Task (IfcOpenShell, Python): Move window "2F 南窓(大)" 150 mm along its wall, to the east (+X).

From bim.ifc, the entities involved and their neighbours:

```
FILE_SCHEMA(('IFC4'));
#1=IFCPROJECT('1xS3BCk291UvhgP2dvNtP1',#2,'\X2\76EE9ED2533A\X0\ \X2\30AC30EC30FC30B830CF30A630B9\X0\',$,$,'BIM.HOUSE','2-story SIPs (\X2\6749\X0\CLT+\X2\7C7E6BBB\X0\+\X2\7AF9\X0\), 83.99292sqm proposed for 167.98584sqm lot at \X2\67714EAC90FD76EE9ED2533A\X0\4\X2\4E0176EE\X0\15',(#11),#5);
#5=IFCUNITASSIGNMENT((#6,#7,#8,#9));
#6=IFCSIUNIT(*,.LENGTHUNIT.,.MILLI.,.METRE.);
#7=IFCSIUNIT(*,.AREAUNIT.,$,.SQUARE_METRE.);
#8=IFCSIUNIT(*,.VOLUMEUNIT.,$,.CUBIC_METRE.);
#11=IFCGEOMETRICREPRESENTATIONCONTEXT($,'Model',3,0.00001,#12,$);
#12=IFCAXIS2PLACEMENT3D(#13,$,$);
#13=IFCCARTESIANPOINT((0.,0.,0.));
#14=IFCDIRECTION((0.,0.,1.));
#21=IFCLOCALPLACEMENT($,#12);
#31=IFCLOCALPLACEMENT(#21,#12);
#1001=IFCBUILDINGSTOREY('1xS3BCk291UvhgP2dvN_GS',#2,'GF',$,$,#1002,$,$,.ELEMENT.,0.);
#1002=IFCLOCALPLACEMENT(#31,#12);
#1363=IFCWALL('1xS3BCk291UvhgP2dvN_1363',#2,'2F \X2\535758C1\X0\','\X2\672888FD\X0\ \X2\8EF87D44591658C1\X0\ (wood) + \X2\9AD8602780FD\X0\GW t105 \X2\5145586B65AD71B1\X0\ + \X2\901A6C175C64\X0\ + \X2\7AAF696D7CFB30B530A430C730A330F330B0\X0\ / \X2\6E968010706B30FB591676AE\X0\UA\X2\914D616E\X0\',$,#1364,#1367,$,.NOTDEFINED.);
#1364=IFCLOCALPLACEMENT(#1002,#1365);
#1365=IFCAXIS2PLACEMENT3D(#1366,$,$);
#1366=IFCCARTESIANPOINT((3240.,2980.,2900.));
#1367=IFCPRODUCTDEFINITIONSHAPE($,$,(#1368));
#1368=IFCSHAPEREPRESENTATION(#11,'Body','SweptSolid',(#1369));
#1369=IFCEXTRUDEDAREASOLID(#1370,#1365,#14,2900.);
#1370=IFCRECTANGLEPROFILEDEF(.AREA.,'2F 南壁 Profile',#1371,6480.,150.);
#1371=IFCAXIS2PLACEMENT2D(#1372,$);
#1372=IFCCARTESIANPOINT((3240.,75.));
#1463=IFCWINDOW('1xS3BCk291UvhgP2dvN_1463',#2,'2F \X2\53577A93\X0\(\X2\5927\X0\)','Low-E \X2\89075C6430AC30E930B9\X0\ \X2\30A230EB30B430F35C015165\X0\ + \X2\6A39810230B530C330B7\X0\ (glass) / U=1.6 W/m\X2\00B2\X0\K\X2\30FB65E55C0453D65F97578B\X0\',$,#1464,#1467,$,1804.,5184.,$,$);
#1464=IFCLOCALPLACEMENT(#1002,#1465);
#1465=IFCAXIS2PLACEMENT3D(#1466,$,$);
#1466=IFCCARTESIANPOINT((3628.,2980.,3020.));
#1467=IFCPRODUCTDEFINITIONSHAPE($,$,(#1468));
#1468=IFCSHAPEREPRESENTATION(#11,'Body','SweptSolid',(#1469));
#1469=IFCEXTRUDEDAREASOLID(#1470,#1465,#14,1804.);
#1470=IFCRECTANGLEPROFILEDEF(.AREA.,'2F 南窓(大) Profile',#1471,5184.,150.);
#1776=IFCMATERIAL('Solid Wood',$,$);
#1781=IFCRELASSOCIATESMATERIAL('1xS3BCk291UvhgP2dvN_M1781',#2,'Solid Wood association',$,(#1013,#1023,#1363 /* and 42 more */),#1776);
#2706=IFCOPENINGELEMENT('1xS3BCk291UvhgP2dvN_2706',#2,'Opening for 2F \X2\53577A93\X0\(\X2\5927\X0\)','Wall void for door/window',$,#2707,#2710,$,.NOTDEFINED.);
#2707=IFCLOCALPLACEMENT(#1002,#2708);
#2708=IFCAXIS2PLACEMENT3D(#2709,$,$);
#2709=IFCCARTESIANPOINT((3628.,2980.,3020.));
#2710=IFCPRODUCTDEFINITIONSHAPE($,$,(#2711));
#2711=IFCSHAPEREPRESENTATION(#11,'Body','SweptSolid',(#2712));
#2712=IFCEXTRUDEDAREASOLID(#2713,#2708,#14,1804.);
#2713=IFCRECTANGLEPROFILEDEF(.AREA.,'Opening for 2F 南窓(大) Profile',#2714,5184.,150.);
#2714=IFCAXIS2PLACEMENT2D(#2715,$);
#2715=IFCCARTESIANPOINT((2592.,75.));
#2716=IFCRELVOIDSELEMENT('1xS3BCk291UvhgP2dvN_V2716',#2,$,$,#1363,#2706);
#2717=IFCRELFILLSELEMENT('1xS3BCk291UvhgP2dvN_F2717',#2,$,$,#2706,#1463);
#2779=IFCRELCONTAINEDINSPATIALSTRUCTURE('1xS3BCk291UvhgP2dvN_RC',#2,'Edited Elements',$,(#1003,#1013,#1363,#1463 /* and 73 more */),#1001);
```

```python
import ifcopenshell
import ifcopenshell.api.geometry
import ifcopenshell.util.placement
import ifcopenshell.util.unit

model = ifcopenshell.open("bim.ifc")
unit_scale = ifcopenshell.util.unit.calculate_unit_scale(model)

window = model.by_guid("1xS3BCk291UvhgP2dvN_1463")
opening = window.FillsVoids[0].RelatingOpeningElement
wall = opening.VoidsElements[0].RelatingBuildingElement

wall_matrix = ifcopenshell.util.placement.get_local_placement(wall.ObjectPlacement)
shift = wall_matrix[:3, 0] * 0.15 / unit_scale
before = ifcopenshell.util.placement.get_local_placement(window.ObjectPlacement)[:3, 3].copy()

# The window is not placed relative to its opening, so move both.
for product in (opening, window):
    matrix = ifcopenshell.util.placement.get_local_placement(product.ObjectPlacement)
    matrix[:3, 3] += shift
    ifcopenshell.api.geometry.edit_object_placement(model, product=product, matrix=matrix, is_si=False)

after = ifcopenshell.util.placement.get_local_placement(window.ObjectPlacement)[:3, 3]
print("window moved by", (after - before).round(3) + 0.0)

model.write("bim_edited.ifc")
```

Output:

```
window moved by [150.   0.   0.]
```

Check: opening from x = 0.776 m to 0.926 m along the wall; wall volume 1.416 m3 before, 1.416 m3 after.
